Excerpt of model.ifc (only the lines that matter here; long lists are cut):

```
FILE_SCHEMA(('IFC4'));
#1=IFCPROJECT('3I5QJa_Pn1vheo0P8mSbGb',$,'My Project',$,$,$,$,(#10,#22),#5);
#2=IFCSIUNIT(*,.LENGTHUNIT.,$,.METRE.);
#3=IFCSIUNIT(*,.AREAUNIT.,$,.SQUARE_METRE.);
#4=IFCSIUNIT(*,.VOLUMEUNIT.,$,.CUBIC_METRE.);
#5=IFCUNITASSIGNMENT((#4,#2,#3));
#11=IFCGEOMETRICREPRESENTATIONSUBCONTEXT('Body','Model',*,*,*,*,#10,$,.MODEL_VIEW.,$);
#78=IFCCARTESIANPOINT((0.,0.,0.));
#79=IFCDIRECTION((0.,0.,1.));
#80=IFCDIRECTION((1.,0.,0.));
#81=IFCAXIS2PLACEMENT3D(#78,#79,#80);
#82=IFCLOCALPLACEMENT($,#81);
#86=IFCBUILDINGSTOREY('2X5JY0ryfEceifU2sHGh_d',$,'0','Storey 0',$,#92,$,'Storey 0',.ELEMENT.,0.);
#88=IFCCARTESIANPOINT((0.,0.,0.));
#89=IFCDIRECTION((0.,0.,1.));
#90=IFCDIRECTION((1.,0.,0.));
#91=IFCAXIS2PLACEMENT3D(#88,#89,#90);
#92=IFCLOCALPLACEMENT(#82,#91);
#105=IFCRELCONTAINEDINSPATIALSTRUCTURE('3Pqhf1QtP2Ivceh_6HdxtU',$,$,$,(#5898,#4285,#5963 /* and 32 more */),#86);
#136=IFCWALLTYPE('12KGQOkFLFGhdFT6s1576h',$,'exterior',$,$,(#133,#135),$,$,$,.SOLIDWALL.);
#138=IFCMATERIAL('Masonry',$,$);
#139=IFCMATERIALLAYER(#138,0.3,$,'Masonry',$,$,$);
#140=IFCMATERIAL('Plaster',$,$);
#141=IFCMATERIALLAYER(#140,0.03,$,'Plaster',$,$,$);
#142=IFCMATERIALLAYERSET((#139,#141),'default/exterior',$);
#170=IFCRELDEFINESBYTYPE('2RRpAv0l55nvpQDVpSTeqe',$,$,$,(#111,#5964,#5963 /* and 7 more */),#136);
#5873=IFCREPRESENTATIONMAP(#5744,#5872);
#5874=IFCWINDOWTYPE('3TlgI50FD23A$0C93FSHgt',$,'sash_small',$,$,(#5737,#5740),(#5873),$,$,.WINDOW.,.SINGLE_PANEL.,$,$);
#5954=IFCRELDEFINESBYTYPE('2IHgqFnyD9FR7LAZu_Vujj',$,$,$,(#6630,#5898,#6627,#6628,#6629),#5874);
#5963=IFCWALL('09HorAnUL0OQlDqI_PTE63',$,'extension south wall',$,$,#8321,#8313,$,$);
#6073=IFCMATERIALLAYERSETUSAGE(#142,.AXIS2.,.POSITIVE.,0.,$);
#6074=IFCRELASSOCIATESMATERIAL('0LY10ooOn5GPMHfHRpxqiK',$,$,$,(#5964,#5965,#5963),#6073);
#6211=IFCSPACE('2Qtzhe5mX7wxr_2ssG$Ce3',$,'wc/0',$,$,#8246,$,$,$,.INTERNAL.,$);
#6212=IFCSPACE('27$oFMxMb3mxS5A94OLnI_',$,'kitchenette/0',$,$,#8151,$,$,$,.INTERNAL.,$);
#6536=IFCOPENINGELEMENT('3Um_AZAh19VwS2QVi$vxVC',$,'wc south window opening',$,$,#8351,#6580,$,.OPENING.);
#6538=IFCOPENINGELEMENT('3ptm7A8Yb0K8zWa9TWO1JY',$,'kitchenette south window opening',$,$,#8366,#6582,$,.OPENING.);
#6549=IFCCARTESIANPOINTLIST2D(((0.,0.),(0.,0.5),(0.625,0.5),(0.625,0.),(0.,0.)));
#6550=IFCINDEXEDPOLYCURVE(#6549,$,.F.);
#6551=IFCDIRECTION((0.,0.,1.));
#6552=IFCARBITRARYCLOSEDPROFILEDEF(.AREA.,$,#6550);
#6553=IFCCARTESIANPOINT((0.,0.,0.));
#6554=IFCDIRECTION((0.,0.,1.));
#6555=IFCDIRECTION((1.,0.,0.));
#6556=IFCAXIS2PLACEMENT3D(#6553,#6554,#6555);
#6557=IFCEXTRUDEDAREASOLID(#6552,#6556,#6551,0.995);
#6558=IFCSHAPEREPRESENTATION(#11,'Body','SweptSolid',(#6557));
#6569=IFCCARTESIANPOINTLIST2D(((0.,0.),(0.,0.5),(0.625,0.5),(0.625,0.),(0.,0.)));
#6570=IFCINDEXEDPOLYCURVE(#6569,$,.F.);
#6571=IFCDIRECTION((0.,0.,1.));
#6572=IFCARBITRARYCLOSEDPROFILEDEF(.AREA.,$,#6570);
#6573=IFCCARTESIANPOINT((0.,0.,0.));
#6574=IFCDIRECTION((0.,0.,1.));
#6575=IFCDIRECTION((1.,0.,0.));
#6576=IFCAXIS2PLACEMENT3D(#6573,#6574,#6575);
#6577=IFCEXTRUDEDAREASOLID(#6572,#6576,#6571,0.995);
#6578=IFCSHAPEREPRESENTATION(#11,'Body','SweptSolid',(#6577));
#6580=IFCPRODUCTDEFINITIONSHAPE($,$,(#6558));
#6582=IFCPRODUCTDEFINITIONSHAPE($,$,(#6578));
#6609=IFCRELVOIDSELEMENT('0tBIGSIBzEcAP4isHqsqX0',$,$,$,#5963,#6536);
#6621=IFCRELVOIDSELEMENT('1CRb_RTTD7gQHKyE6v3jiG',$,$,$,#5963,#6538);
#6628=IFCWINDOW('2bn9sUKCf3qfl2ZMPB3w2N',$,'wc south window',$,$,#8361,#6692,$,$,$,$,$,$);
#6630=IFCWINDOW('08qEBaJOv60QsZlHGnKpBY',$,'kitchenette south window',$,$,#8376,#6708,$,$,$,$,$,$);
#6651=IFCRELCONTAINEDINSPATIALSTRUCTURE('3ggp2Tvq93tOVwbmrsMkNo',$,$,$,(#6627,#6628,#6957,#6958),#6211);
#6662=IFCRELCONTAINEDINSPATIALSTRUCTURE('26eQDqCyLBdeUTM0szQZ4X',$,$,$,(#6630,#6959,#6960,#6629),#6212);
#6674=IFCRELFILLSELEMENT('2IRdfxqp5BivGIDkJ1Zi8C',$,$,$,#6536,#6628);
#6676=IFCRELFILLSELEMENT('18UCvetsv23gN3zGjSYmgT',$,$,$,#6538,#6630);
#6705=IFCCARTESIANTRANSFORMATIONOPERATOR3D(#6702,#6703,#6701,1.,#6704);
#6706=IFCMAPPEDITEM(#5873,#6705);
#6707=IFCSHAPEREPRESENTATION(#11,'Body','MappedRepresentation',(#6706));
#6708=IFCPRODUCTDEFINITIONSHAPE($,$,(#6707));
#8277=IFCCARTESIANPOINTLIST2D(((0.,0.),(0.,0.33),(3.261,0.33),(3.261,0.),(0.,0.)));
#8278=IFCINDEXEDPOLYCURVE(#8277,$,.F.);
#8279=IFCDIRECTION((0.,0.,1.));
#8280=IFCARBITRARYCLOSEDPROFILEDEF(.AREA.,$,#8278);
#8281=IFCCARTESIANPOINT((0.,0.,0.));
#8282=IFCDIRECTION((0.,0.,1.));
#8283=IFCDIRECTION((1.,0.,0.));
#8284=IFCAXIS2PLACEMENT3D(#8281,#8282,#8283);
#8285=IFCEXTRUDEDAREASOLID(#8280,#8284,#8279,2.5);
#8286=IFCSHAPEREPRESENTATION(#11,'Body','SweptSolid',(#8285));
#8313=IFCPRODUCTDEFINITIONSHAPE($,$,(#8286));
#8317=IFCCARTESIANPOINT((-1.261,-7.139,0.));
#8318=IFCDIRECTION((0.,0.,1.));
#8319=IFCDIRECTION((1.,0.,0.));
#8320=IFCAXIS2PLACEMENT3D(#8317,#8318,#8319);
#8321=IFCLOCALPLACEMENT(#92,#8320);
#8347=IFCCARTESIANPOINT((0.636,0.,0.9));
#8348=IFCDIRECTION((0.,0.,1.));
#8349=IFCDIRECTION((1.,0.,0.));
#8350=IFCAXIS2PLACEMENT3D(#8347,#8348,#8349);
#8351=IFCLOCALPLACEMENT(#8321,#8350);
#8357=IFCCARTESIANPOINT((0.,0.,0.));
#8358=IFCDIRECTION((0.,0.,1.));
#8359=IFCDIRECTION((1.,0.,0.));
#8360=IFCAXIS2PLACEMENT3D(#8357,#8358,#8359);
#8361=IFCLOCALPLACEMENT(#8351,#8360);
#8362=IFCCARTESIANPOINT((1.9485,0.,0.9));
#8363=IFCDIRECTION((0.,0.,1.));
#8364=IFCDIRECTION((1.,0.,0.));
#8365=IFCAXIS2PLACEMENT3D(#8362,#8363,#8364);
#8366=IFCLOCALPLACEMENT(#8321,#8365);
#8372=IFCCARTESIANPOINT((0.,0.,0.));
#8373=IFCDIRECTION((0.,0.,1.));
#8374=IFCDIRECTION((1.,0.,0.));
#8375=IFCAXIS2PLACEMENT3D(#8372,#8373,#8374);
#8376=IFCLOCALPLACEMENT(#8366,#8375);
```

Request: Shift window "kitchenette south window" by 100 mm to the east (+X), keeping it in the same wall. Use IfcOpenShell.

```python
import ifcopenshell
import ifcopenshell.api.geometry
import ifcopenshell.util.placement

model = ifcopenshell.open("model.ifc")

window = model.by_guid("08qEBaJOv60QsZlHGnKpBY")
opening = window.FillsVoids[0].RelatingOpeningElement
wall = opening.VoidsElements[0].RelatingBuildingElement

wall_matrix = ifcopenshell.util.placement.get_local_placement(wall.ObjectPlacement)
shift = wall_matrix[:3, 0] * 0.1
before = ifcopenshell.util.placement.get_local_placement(window.ObjectPlacement)[:3, 3].copy()

# The window is placed relative to its opening, so it follows when the opening moves.
matrix = ifcopenshell.util.placement.get_local_placement(opening.ObjectPlacement)
matrix[:3, 3] += shift
ifcopenshell.api.geometry.edit_object_placement(
    model, product=opening, matrix=matrix, is_si=False, should_transform_children=True
)

after = ifcopenshell.util.placement.get_local_placement(window.ObjectPlacement)[:3, 3]
print("window moved by", (after - before).round(3) + 0.0)

model.write("model_rev.ifc")
```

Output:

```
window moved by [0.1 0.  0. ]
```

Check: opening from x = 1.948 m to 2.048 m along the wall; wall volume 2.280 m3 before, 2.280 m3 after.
